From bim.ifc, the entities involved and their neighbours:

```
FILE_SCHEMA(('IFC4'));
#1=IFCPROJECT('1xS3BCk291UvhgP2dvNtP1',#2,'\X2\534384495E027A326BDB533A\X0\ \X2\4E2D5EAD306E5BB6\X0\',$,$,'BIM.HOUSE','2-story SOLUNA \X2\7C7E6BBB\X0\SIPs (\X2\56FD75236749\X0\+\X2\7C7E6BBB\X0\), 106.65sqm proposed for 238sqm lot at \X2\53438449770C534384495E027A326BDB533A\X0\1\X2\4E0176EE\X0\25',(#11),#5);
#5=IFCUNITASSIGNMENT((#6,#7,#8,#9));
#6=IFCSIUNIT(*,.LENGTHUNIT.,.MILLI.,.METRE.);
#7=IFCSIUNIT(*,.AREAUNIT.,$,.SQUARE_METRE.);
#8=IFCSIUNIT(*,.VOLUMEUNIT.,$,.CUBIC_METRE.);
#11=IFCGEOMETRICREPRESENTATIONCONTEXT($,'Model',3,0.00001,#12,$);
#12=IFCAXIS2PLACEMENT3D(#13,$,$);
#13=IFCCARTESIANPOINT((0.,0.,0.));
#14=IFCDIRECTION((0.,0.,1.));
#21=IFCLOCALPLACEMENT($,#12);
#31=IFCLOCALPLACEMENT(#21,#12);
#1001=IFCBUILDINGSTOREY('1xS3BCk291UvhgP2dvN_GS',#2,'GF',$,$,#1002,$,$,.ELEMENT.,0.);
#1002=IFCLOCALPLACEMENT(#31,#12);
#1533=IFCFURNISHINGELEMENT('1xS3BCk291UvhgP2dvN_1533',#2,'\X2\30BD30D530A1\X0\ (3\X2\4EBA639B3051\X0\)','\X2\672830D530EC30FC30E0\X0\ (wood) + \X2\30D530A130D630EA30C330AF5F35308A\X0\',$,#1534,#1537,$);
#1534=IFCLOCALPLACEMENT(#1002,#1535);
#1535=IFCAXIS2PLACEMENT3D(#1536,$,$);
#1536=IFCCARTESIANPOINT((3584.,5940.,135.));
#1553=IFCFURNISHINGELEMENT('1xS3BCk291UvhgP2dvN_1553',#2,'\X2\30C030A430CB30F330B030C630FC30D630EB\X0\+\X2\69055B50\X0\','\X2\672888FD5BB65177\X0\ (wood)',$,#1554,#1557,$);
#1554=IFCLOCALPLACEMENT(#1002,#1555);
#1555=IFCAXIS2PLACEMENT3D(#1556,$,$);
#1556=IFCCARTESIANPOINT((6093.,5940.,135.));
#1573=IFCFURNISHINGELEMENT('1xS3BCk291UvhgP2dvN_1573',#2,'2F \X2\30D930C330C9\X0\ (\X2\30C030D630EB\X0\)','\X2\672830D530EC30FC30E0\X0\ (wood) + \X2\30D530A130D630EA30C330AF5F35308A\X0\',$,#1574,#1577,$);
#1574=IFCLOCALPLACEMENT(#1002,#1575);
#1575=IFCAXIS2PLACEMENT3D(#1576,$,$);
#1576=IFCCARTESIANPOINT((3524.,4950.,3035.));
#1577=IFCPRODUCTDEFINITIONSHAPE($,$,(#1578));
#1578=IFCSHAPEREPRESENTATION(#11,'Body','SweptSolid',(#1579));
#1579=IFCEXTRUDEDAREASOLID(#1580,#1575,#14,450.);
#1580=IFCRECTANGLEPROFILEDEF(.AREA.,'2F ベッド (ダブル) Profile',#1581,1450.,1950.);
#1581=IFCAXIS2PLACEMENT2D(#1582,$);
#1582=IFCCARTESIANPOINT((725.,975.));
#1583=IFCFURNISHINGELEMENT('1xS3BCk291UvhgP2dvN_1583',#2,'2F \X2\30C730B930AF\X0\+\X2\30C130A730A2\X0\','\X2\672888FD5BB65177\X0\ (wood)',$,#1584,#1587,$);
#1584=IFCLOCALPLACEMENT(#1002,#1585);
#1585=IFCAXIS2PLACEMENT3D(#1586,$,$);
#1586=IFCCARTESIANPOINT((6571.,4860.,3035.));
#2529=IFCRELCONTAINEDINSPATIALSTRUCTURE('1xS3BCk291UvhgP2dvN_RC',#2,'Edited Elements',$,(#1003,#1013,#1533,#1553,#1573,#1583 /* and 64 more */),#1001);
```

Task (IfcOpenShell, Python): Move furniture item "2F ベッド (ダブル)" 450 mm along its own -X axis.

```python
import ifcopenshell
import ifcopenshell.api.geometry
import ifcopenshell.util.placement
import ifcopenshell.util.unit

model = ifcopenshell.open("bim.ifc")
unit_scale = ifcopenshell.util.unit.calculate_unit_scale(model)

item = model.by_guid("1xS3BCk291UvhgP2dvN_1573")
matrix = ifcopenshell.util.placement.get_local_placement(item.ObjectPlacement)
matrix[:3, 3] -= matrix[:3, 0] * 0.45 / unit_scale
ifcopenshell.api.geometry.edit_object_placement(model, product=item, matrix=matrix, is_si=False)

print(ifcopenshell.util.placement.get_local_placement(item.ObjectPlacement).round(3) + 0.0)

model.write("bim_rev.ifc")
```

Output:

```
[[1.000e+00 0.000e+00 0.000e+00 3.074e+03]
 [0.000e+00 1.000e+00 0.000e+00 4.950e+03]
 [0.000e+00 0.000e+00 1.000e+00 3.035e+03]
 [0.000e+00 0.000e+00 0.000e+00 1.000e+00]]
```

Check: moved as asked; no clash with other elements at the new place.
